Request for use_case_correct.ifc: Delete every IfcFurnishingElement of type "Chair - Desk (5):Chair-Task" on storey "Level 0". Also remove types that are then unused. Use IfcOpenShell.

First a look at what the model holds.

```python
import ifcopenshell
import ifcopenshell.util.element

model = ifcopenshell.open("use_case_correct.ifc")
print(model.schema)
storey = next(s for s in model.by_type("IfcBuildingStorey") if s.Name == "Level 0")
furniture = [e for e in ifcopenshell.util.element.get_decomposition(storey) if e.is_a("IfcFurnishingElement")]
seen = {}
for e in furniture:
    element_type = ifcopenshell.util.element.get_type(e)
    name = element_type.Name if element_type not in (None, e) else None
    seen[name] = seen.get(name, 0) + 1
for name, count in sorted(seen.items(), key=str):
    print(count, "x", name)
```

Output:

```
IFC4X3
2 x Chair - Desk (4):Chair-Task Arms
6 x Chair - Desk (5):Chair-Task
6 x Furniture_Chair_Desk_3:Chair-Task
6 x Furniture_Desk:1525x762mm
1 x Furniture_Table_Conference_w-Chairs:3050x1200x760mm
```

```python
import ifcopenshell
import ifcopenshell.api.root
import ifcopenshell.util.element

model = ifcopenshell.open("use_case_correct.ifc")

storey = next(s for s in model.by_type("IfcBuildingStorey") if s.Name == "Level 0")
furniture = [e for e in ifcopenshell.util.element.get_decomposition(storey) if e.is_a("IfcFurnishingElement")]
targets = [e for e in furniture if (t := ifcopenshell.util.element.get_type(e)) not in (None, e) and t.Name == "Chair - Desk (5):Chair-Task"]
types = {ifcopenshell.util.element.get_type(e) for e in targets} - {None, *targets}

for e in targets:
    ifcopenshell.api.root.remove_product(model, product=e)
print(len(targets), "removed")

unused = [t for t in types if not ifcopenshell.util.element.get_types(t)]
for t in unused:
    ifcopenshell.api.root.remove_product(model, product=t)
print(len(unused), "unused types removed")

model.write("use_case_correct_rev.ifc")
```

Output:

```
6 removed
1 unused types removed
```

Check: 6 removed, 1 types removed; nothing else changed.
